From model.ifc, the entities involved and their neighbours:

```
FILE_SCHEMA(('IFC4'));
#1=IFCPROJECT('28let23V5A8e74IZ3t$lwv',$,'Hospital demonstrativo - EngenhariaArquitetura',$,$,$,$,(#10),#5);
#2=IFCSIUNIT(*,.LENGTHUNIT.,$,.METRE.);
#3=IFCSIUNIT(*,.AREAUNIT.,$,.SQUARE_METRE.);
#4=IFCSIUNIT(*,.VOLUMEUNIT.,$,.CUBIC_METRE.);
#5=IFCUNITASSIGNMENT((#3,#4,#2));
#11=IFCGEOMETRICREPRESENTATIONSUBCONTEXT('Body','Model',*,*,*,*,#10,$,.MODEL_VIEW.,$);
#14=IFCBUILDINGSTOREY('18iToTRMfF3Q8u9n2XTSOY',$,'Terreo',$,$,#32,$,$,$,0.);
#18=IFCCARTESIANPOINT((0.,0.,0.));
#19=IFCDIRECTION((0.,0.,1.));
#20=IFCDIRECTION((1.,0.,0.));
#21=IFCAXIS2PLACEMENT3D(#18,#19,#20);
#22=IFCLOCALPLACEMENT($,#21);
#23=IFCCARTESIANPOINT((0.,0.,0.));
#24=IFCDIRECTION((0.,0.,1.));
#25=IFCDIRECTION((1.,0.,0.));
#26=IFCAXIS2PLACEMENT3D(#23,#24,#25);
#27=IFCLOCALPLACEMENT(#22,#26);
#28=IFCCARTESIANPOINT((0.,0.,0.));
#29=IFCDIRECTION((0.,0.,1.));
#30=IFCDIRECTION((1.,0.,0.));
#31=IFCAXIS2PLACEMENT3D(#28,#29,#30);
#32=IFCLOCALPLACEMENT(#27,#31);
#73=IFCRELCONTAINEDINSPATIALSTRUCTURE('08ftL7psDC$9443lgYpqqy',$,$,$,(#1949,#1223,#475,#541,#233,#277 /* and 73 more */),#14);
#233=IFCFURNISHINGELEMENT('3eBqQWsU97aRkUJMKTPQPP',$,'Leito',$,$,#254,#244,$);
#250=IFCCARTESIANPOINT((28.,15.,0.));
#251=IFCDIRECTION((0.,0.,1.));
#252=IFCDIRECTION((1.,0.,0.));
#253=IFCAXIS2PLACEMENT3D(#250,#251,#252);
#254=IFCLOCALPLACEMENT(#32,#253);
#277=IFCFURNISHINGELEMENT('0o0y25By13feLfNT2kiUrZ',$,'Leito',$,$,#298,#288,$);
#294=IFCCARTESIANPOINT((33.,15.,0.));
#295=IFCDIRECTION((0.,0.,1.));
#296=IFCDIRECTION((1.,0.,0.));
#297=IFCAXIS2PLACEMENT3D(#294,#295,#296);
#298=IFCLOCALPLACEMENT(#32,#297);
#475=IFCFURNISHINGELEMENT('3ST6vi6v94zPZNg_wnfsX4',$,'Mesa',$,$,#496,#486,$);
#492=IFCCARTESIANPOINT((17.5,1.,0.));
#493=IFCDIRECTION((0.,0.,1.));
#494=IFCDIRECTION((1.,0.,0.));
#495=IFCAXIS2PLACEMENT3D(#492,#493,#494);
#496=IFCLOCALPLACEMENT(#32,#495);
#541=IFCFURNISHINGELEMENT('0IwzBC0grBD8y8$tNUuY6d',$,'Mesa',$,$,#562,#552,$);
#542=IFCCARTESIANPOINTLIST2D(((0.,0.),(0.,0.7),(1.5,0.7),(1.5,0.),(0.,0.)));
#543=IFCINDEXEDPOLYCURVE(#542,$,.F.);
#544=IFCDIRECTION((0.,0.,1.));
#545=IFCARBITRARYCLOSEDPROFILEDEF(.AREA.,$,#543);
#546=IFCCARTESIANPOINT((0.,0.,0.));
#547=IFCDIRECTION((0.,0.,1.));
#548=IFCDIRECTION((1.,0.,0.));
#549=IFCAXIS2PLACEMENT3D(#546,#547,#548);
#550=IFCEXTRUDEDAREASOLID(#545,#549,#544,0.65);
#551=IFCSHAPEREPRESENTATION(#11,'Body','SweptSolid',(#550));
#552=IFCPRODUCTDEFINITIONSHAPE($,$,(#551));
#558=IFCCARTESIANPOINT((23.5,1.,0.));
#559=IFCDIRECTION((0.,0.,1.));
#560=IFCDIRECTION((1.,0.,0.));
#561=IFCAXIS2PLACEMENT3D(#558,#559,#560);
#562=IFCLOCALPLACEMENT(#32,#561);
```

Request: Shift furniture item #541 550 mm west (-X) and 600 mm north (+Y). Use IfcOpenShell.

```python
import ifcopenshell
import ifcopenshell.api.geometry
import ifcopenshell.util.placement

model = ifcopenshell.open("model.ifc")

item = model.by_guid("0IwzBC0grBD8y8$tNUuY6d")
matrix = ifcopenshell.util.placement.get_local_placement(item.ObjectPlacement)
matrix[0, 3] -= 0.55
matrix[1, 3] += 0.6
ifcopenshell.api.geometry.edit_object_placement(model, product=item, matrix=matrix, is_si=False)

print(ifcopenshell.util.placement.get_local_placement(item.ObjectPlacement).round(3) + 0.0)

model.write("model_edited.ifc")
```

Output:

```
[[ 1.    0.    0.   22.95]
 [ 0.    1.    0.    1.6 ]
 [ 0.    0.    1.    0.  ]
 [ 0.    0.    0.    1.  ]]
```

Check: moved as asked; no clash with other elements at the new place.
